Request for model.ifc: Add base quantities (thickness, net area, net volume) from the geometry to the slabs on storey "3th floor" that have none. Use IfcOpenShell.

First a look at what the model holds.

```python
import ifcopenshell
import ifcopenshell.util.element
import ifcopenshell.util.unit

model = ifcopenshell.open("model.ifc")
print(model.schema)
for unit_type in ("LENGTHUNIT", "AREAUNIT", "VOLUMEUNIT"):
    print(unit_type, ifcopenshell.util.unit.calculate_unit_scale(model, unit_type))
storey = next(s for s in model.by_type("IfcBuildingStorey") if s.Name == "3th floor")
slabs = [e for e in ifcopenshell.util.element.get_decomposition(storey) if e.is_a("IfcSlab")]
for e in sorted(slabs, key=lambda e: e.id()):
    print(e.id(), e.is_a(), e.Name, list(ifcopenshell.util.element.get_psets(e, qtos_only=True)), sep=" | ")
```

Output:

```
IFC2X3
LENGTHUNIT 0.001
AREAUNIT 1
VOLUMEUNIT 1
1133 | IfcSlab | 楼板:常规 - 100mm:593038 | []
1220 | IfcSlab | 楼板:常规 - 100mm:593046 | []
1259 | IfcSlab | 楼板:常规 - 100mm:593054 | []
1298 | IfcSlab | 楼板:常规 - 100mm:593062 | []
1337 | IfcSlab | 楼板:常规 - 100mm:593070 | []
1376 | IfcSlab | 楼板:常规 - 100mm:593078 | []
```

```python
import ifcopenshell
import ifcopenshell.api.pset
import ifcopenshell.geom
import ifcopenshell.util.element
import ifcopenshell.util.shape
import ifcopenshell.util.unit

model = ifcopenshell.open("model.ifc")
unit_scale = ifcopenshell.util.unit.calculate_unit_scale(model)
area_scale = ifcopenshell.util.unit.calculate_unit_scale(model, "AREAUNIT")
volume_scale = ifcopenshell.util.unit.calculate_unit_scale(model, "VOLUMEUNIT")
settings = ifcopenshell.geom.settings()

storey = next(s for s in model.by_type("IfcBuildingStorey") if s.Name == "3th floor")
slabs = [e for e in ifcopenshell.util.element.get_decomposition(storey) if e.is_a("IfcSlab")]

for e in sorted(slabs, key=lambda e: e.id()):
    if ifcopenshell.util.element.get_psets(e, qtos_only=True, should_inherit=False):
        continue
    # Geometry comes back in metres, in the element's own axes.
    shape = ifcopenshell.geom.create_shape(settings, e)
    values = {
        "Width": ifcopenshell.util.shape.get_z(shape.geometry) / unit_scale,
        "NetArea": ifcopenshell.util.shape.get_footprint_area(shape.geometry) / area_scale,
        "NetVolume": ifcopenshell.util.shape.get_volume(shape.geometry) / volume_scale,
    }
    qto = ifcopenshell.api.pset.add_qto(model, product=e, name="BaseQuantities")
    ifcopenshell.api.pset.edit_qto(model, qto=qto, properties=values)
    print(e.id(), {k: round(v, 3) for k, v in values.items()})

model.write("model_updated.ifc")
```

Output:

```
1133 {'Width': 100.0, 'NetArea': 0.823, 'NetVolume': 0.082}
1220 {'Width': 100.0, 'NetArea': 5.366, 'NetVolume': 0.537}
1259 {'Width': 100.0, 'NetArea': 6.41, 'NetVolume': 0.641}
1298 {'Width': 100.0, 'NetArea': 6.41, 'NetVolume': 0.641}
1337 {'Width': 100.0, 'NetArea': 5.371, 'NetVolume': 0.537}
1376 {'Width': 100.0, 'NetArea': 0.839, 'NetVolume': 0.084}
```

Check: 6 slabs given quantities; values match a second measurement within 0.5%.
